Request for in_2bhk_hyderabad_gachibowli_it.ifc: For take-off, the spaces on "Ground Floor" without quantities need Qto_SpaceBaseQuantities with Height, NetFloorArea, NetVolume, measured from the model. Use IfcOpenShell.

First a look at what the model holds.

```python
import ifcopenshell
import ifcopenshell.util.element
import ifcopenshell.util.unit

model = ifcopenshell.open("in_2bhk_hyderabad_gachibowli_it.ifc")
print(model.schema)
for unit_type in ("LENGTHUNIT", "AREAUNIT", "VOLUMEUNIT"):
    print(unit_type, ifcopenshell.util.unit.calculate_unit_scale(model, unit_type))
storey = next(s for s in model.by_type("IfcBuildingStorey") if s.Name == "Ground Floor")
spaces = [e for e in ifcopenshell.util.element.get_decomposition(storey) if e.is_a("IfcSpace")]
for e in sorted(spaces, key=lambda e: e.id()):
    print(e.id(), e.is_a(), e.Name, list(ifcopenshell.util.element.get_psets(e, qtos_only=True)), sep=" | ")
```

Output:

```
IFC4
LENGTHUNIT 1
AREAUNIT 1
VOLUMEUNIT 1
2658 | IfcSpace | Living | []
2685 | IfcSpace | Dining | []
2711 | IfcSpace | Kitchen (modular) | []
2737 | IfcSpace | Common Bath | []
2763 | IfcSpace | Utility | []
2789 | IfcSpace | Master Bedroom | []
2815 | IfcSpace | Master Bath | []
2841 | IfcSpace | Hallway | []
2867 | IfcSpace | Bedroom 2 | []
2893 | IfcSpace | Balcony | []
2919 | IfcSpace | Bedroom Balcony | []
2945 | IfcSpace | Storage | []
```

```python
import ifcopenshell
import ifcopenshell.api.pset
import ifcopenshell.geom
import ifcopenshell.util.element
import ifcopenshell.util.shape
import ifcopenshell.util.unit

model = ifcopenshell.open("in_2bhk_hyderabad_gachibowli_it.ifc")
unit_scale = ifcopenshell.util.unit.calculate_unit_scale(model)
area_scale = ifcopenshell.util.unit.calculate_unit_scale(model, "AREAUNIT")
volume_scale = ifcopenshell.util.unit.calculate_unit_scale(model, "VOLUMEUNIT")
settings = ifcopenshell.geom.settings()

storey = next(s for s in model.by_type("IfcBuildingStorey") if s.Name == "Ground Floor")
spaces = [e for e in ifcopenshell.util.element.get_decomposition(storey) if e.is_a("IfcSpace")]

for e in sorted(spaces, key=lambda e: e.id()):
    if ifcopenshell.util.element.get_psets(e, qtos_only=True, should_inherit=False):
        continue
    # Geometry comes back in metres, in the element's own axes.
    shape = ifcopenshell.geom.create_shape(settings, e)
    values = {
        "Height": ifcopenshell.util.shape.get_z(shape.geometry) / unit_scale,
        "NetFloorArea": ifcopenshell.util.shape.get_footprint_area(shape.geometry) / area_scale,
        "NetVolume": ifcopenshell.util.shape.get_volume(shape.geometry) / volume_scale,
    }
    qto = ifcopenshell.api.pset.add_qto(model, product=e, name="Qto_SpaceBaseQuantities")
    ifcopenshell.api.pset.edit_qto(model, qto=qto, properties=values)
    print(e.id(), {k: round(v, 3) for k, v in values.items()})

model.write("in_2bhk_hyderabad_gachibowli_it_rev.ifc")
```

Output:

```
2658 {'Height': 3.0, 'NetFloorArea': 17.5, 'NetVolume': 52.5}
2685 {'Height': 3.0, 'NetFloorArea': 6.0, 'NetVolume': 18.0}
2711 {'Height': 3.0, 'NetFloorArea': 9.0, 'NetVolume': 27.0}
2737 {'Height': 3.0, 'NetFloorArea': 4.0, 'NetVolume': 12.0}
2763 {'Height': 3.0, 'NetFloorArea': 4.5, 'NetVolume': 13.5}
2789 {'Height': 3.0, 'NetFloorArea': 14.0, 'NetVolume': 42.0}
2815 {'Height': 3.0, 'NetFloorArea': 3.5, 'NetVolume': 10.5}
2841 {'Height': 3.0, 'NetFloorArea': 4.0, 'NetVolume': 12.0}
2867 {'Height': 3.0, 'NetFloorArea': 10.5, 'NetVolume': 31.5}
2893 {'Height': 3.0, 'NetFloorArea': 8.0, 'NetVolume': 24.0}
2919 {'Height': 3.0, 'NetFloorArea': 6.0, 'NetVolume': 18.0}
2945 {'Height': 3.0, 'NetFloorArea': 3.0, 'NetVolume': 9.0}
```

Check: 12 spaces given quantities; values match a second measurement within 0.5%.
